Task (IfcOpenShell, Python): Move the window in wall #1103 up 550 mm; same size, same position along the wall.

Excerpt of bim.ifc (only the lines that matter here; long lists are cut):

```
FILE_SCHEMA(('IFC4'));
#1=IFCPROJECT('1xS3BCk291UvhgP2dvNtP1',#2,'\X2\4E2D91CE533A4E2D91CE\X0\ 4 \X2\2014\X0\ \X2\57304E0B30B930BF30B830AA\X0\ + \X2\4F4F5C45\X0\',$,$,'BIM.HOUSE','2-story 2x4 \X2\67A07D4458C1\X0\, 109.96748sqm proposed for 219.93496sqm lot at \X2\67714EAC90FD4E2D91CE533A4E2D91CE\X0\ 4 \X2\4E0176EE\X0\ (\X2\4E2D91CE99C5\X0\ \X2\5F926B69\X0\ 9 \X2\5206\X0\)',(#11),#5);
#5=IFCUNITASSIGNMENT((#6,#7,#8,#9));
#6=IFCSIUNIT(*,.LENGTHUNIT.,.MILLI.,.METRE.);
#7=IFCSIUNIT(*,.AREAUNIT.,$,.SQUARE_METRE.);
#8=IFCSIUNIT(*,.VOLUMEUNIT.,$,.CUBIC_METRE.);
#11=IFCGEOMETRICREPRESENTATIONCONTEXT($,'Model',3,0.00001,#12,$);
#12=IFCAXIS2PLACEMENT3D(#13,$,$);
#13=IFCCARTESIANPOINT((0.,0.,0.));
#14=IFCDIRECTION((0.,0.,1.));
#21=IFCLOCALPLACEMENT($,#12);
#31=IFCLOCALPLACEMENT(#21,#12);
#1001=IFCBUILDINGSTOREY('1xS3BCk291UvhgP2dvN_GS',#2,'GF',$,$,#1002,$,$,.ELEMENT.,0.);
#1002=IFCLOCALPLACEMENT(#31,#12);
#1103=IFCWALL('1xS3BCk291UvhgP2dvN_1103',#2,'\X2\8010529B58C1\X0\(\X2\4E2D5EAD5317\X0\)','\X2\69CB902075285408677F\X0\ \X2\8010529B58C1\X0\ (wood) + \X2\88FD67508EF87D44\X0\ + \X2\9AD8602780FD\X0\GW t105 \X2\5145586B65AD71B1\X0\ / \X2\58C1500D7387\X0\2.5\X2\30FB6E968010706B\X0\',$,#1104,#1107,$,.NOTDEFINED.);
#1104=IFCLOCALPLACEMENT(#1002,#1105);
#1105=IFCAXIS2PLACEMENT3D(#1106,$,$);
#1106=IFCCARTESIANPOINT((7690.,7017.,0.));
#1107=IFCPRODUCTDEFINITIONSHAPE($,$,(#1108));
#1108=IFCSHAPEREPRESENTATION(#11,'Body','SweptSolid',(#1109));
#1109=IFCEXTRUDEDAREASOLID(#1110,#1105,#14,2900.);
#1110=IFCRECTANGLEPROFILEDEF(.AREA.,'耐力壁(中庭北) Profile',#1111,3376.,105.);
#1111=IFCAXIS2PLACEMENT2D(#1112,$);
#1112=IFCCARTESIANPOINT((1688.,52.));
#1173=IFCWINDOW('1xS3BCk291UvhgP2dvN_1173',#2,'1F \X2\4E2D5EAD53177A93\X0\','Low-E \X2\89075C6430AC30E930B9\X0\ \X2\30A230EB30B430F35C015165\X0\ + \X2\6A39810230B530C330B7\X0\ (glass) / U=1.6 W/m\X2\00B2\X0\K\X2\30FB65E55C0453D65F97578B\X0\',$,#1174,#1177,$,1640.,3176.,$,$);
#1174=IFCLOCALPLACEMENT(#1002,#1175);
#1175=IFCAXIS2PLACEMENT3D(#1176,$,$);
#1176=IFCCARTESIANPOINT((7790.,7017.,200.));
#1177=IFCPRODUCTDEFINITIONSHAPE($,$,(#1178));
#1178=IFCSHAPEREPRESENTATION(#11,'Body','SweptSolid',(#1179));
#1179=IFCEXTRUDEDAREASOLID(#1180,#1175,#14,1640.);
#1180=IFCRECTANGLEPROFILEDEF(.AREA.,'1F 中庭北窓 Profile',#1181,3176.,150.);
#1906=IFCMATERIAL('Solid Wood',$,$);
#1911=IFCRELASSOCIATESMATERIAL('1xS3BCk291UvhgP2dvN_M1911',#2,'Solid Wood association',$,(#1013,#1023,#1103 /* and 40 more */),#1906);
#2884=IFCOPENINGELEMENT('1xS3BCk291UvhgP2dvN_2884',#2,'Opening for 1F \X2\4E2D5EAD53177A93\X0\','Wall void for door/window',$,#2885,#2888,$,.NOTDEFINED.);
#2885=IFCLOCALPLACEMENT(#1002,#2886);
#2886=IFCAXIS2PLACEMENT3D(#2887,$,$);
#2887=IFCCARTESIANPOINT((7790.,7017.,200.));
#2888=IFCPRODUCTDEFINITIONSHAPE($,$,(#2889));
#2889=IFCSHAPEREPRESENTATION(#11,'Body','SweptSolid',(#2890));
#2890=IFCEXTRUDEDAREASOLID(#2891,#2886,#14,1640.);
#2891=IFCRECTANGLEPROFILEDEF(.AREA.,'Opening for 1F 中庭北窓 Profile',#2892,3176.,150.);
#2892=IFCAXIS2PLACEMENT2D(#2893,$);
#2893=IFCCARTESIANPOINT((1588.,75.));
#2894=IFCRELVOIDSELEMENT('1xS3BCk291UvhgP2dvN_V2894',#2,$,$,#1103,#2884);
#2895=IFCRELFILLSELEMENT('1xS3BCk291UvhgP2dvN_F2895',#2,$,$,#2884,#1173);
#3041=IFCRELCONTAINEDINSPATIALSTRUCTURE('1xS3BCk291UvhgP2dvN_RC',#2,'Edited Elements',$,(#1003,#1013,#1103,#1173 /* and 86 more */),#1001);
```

```python
import numpy as np
import ifcopenshell
import ifcopenshell.api.geometry
import ifcopenshell.util.placement
import ifcopenshell.util.unit

model = ifcopenshell.open("bim.ifc")
unit_scale = ifcopenshell.util.unit.calculate_unit_scale(model)

window = model.by_guid("1xS3BCk291UvhgP2dvN_1173")
opening = window.FillsVoids[0].RelatingOpeningElement
dz = 550.0

shift = np.array([0.0, 0.0, dz])
# The window is not placed relative to its opening, so move both.
for product in (opening, window):
    matrix = ifcopenshell.util.placement.get_local_placement(product.ObjectPlacement)
    matrix[:3, 3] += shift
    ifcopenshell.api.geometry.edit_object_placement(model, product=product, matrix=matrix, is_si=False)

print(f"moved by {dz * unit_scale:+.3f} m")

model.write("bim_v2.ifc")
```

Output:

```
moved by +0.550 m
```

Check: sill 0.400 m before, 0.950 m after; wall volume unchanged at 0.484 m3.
